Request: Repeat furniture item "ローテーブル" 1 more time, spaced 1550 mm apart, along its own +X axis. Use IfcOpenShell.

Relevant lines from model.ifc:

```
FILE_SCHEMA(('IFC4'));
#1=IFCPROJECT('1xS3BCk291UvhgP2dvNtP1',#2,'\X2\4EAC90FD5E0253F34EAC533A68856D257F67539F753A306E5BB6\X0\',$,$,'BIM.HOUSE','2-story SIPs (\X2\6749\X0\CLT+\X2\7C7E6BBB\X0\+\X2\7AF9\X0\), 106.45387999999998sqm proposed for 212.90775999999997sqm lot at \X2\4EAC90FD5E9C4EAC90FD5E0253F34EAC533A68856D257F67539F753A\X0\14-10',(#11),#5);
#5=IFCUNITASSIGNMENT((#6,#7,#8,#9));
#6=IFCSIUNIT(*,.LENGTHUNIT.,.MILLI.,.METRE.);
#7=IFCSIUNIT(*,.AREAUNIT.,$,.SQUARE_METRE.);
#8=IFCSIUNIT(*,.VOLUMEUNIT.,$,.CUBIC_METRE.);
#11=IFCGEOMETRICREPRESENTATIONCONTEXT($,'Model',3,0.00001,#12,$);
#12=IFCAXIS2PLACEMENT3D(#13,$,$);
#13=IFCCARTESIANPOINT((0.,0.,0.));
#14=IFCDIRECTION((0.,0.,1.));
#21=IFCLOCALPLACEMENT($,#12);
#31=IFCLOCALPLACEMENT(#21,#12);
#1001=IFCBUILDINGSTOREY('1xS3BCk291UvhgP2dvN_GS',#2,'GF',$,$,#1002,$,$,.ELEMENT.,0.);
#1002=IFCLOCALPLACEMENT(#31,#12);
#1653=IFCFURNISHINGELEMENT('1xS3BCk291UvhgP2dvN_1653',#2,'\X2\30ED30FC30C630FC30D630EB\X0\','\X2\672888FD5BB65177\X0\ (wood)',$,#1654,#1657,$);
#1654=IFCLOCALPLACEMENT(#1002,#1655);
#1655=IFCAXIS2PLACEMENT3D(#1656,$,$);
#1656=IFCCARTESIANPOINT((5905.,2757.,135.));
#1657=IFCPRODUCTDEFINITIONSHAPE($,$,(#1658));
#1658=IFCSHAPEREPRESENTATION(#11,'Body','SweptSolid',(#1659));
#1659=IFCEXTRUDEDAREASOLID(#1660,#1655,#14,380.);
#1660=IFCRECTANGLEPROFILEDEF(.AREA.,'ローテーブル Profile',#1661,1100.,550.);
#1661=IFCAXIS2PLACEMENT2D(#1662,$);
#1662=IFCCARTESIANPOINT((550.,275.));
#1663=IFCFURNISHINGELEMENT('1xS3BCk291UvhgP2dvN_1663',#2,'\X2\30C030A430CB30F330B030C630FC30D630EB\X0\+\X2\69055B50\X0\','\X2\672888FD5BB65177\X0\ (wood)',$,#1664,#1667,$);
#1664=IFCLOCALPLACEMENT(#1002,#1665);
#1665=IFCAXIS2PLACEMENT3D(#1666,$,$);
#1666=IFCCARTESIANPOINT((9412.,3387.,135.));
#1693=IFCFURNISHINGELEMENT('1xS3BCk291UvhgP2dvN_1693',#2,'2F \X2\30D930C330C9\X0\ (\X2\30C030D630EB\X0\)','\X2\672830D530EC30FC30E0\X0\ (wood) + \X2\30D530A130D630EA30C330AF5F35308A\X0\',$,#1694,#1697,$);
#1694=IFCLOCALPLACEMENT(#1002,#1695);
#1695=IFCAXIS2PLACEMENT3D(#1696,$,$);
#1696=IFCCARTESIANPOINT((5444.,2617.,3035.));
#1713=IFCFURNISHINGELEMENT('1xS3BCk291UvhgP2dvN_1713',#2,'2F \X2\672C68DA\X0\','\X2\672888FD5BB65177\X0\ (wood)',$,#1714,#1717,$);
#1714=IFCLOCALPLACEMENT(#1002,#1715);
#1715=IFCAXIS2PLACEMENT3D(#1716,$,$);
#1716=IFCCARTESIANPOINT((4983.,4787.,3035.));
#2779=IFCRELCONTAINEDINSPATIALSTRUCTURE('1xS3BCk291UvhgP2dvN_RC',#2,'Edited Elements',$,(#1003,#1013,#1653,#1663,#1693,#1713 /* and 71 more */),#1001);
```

```python
import ifcopenshell
import ifcopenshell.api.geometry
import ifcopenshell.api.root
import ifcopenshell.util.element
import ifcopenshell.util.placement
import ifcopenshell.util.unit

model = ifcopenshell.open("model.ifc")
unit_scale = ifcopenshell.util.unit.calculate_unit_scale(model)


def reuse_history(source, copy):
    """copy_class also copies each property set's owner history, people and application; keep the originals."""
    for rel in copy.IsDefinedBy:
        if rel.is_a("IfcRelDefinesByProperties") and (history := rel.RelatingPropertyDefinition.OwnerHistory):
            rel.RelatingPropertyDefinition.OwnerHistory = source.OwnerHistory
            ifcopenshell.util.element.remove_deep2(model, history)


source = model.by_guid("1xS3BCk291UvhgP2dvN_1653")
base = ifcopenshell.util.placement.get_local_placement(source.ObjectPlacement)
step = base[:3, 0] * 1.55 / unit_scale

for i in range(1, 2):
    copy = ifcopenshell.api.root.copy_class(model, product=source)
    copy.Representation = ifcopenshell.util.element.copy_deep(
        model, source.Representation, exclude=["IfcGeometricRepresentationContext", "IfcRepresentationMap"]
    )
    reuse_history(source, copy)
    matrix = base.copy()
    matrix[:3, 3] += i * step
    print("added at", matrix[:3, 3].round(3) + 0.0)
    ifcopenshell.api.geometry.edit_object_placement(model, product=copy, matrix=matrix, is_si=False)

model.write("model_rev.ifc")
```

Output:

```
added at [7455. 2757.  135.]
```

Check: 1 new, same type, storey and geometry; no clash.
